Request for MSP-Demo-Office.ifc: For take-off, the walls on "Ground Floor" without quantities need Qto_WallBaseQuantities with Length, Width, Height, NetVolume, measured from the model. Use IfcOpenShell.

First a look at what the model holds.

```python
import ifcopenshell
import ifcopenshell.util.element
import ifcopenshell.util.unit

model = ifcopenshell.open("MSP-Demo-Office.ifc")
print(model.schema)
for unit_type in ("LENGTHUNIT", "AREAUNIT", "VOLUMEUNIT"):
    print(unit_type, ifcopenshell.util.unit.calculate_unit_scale(model, unit_type))
storey = next(s for s in model.by_type("IfcBuildingStorey") if s.Name == "Ground Floor")
walls = [e for e in ifcopenshell.util.element.get_decomposition(storey) if e.is_a("IfcWall")]
for e in sorted(walls, key=lambda e: e.id()):
    print(e.id(), e.is_a(), e.Name, list(ifcopenshell.util.element.get_psets(e, qtos_only=True)), sep=" | ")
```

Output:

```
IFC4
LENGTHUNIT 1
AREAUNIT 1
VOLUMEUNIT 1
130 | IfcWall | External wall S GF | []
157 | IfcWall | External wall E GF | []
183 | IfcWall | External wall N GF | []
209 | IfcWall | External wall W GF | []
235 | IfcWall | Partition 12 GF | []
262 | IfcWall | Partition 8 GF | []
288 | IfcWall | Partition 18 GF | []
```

```python
import ifcopenshell
import ifcopenshell.api.pset
import ifcopenshell.geom
import ifcopenshell.util.element
import ifcopenshell.util.shape
import ifcopenshell.util.unit

model = ifcopenshell.open("MSP-Demo-Office.ifc")
unit_scale = ifcopenshell.util.unit.calculate_unit_scale(model)
volume_scale = ifcopenshell.util.unit.calculate_unit_scale(model, "VOLUMEUNIT")
settings = ifcopenshell.geom.settings()

storey = next(s for s in model.by_type("IfcBuildingStorey") if s.Name == "Ground Floor")
walls = [e for e in ifcopenshell.util.element.get_decomposition(storey) if e.is_a("IfcWall")]

for e in sorted(walls, key=lambda e: e.id()):
    if ifcopenshell.util.element.get_psets(e, qtos_only=True, should_inherit=False):
        continue
    # Geometry comes back in metres, in the element's own axes.
    shape = ifcopenshell.geom.create_shape(settings, e)
    values = {
        "Length": ifcopenshell.util.shape.get_x(shape.geometry) / unit_scale,
        "Width": ifcopenshell.util.shape.get_y(shape.geometry) / unit_scale,
        "Height": ifcopenshell.util.shape.get_z(shape.geometry) / unit_scale,
        "NetVolume": ifcopenshell.util.shape.get_volume(shape.geometry) / volume_scale,
    }
    qto = ifcopenshell.api.pset.add_qto(model, product=e, name="Qto_WallBaseQuantities")
    ifcopenshell.api.pset.edit_qto(model, qto=qto, properties=values)
    print(e.id(), {k: round(v, 3) for k, v in values.items()})

model.write("MSP-Demo-Office_rev.ifc")
```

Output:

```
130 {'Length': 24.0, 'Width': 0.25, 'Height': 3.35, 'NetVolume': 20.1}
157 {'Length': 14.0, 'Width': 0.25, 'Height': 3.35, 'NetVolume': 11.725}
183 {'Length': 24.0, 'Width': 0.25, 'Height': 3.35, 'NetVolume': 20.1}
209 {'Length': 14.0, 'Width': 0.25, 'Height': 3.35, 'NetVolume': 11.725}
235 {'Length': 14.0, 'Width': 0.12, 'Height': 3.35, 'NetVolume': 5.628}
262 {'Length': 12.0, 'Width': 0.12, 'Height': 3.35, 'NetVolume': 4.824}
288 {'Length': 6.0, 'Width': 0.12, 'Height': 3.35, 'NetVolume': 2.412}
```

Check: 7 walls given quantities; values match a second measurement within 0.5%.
